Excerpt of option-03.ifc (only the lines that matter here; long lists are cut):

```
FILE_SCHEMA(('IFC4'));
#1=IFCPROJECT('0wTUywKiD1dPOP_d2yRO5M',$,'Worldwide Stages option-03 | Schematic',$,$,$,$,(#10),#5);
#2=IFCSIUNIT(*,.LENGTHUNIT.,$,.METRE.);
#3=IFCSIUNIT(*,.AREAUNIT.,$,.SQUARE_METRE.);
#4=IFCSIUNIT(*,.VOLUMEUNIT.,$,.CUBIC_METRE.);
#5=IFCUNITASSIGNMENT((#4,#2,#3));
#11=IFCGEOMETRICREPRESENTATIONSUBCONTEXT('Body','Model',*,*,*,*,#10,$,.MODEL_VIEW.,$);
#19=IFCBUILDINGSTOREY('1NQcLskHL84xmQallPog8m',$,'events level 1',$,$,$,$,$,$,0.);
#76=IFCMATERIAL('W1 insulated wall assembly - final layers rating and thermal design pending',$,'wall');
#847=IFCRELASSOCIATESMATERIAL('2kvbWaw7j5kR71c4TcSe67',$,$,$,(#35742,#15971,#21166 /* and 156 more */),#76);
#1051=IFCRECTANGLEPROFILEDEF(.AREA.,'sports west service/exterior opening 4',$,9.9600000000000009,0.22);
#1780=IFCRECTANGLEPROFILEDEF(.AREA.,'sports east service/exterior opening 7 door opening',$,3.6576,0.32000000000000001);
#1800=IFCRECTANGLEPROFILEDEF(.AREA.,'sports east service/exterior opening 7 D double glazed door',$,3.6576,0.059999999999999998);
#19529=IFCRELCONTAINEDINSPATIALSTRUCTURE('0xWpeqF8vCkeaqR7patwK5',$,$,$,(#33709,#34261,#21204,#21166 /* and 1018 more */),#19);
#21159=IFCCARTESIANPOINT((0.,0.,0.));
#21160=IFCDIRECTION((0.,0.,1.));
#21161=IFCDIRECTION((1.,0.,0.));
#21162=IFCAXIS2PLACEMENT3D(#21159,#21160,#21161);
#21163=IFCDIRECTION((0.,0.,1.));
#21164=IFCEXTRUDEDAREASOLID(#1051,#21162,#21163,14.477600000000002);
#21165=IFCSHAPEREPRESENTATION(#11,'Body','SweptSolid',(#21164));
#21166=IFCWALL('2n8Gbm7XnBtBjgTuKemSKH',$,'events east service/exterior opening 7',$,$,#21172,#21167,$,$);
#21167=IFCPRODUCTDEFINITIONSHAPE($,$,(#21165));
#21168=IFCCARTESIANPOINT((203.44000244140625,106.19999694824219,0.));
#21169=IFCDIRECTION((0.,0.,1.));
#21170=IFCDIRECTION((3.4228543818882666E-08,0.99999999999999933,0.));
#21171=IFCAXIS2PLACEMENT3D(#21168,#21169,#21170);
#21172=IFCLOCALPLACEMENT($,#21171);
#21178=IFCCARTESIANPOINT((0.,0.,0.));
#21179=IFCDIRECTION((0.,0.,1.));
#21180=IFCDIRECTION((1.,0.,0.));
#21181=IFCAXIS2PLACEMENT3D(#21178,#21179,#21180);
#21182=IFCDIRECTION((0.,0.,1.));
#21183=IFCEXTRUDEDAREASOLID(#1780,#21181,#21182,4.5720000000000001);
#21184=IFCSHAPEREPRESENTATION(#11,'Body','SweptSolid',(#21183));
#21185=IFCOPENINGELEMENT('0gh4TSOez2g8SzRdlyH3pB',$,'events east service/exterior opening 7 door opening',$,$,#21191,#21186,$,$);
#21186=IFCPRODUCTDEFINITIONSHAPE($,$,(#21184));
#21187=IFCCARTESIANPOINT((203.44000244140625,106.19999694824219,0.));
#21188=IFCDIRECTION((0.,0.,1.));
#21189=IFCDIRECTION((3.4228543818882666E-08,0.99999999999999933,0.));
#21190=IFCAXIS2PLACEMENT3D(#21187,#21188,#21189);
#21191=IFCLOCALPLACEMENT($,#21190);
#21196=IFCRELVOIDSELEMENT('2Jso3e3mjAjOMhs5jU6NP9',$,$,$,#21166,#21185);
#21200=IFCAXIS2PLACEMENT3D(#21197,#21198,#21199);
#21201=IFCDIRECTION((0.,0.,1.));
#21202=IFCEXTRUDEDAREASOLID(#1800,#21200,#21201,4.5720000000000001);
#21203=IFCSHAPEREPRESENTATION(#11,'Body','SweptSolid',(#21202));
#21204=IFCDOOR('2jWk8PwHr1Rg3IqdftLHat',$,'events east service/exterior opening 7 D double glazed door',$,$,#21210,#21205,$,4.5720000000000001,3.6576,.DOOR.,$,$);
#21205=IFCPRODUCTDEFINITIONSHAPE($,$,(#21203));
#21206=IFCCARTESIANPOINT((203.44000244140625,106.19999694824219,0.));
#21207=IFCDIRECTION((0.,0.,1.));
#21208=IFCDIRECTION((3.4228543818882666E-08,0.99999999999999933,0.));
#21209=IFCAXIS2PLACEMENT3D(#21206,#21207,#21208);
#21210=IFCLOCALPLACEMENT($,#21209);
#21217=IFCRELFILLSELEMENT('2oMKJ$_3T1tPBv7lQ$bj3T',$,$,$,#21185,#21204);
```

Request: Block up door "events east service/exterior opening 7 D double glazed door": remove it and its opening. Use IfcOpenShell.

```python
import ifcopenshell
import ifcopenshell.api.feature
import ifcopenshell.api.root
import ifcopenshell.geom
import ifcopenshell.util.shape

model = ifcopenshell.open("option-03.ifc")
settings = ifcopenshell.geom.settings()


def volume(element):
    """Net volume in cubic metres, openings subtracted."""
    shape = ifcopenshell.geom.create_shape(settings, element)
    return ifcopenshell.util.shape.get_volume(shape.geometry)


door = model.by_guid("2jWk8PwHr1Rg3IqdftLHat")
opening = door.FillsVoids[0].RelatingOpeningElement
wall = opening.VoidsElements[0].RelatingBuildingElement
before = volume(wall)

ifcopenshell.api.root.remove_product(model, product=door)
ifcopenshell.api.feature.remove_feature(model, feature=opening)

after = volume(wall)

print(f"wall volume {before:.3f} -> {after:.3f} m3")

model.write("option-03_edited.ifc")
```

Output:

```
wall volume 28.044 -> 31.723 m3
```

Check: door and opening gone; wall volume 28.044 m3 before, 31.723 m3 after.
